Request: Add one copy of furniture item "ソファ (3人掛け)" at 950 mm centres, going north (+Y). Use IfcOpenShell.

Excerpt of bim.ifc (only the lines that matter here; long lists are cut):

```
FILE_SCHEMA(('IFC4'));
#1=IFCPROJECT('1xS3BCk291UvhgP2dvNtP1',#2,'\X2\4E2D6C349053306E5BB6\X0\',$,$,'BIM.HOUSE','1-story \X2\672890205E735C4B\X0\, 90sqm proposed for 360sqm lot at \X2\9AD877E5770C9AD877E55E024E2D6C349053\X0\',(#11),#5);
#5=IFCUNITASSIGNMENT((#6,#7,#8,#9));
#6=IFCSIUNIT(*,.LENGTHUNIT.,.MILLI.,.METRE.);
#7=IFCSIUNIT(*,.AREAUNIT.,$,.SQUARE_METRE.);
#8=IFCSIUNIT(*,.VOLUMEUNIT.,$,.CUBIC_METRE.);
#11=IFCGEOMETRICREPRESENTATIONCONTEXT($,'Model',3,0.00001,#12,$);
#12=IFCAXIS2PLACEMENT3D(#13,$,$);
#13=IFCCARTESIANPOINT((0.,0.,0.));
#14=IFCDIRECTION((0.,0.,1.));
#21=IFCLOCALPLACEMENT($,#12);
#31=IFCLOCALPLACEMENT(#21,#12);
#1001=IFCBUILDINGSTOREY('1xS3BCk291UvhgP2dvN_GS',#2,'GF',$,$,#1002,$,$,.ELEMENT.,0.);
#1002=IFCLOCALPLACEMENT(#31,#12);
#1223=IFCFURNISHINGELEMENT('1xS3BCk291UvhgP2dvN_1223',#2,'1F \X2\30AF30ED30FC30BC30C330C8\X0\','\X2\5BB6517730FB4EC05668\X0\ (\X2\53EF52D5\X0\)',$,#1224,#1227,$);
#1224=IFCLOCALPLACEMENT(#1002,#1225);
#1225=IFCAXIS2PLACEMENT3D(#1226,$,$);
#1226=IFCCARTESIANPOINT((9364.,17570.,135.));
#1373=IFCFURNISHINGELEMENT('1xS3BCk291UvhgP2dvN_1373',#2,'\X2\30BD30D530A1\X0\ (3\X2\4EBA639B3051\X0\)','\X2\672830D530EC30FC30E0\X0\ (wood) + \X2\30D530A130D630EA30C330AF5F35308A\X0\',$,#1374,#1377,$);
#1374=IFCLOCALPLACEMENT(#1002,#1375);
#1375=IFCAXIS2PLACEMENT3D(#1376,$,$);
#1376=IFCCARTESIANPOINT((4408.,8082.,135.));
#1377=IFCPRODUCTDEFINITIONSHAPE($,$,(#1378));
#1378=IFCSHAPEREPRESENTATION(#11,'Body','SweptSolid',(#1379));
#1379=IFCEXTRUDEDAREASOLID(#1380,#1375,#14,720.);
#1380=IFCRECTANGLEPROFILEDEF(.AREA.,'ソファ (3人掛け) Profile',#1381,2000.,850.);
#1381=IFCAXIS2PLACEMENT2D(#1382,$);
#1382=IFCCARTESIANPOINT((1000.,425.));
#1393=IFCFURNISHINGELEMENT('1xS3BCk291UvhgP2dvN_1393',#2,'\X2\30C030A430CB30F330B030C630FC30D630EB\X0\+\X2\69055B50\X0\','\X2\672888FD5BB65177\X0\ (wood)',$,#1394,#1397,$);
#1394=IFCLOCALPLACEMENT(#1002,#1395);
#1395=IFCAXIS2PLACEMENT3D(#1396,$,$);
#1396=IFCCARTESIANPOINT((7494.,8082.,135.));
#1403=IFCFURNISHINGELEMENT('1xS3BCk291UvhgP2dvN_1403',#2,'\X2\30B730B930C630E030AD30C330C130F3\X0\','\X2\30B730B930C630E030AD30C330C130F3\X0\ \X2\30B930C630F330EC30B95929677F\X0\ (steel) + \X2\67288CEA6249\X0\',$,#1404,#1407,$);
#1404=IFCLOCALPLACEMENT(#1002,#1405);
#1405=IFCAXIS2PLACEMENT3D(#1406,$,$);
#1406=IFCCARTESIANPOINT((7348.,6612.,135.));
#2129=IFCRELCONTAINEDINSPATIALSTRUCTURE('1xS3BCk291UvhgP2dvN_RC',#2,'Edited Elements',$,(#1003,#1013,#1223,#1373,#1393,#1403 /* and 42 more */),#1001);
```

```python
import numpy as np
import ifcopenshell
import ifcopenshell.api.geometry
import ifcopenshell.api.root
import ifcopenshell.util.element
import ifcopenshell.util.placement
import ifcopenshell.util.unit

model = ifcopenshell.open("bim.ifc")
unit_scale = ifcopenshell.util.unit.calculate_unit_scale(model)


def reuse_history(source, copy):
    """copy_class also copies each property set's owner history, people and application; keep the originals."""
    for rel in copy.IsDefinedBy:
        if rel.is_a("IfcRelDefinesByProperties") and (history := rel.RelatingPropertyDefinition.OwnerHistory):
            rel.RelatingPropertyDefinition.OwnerHistory = source.OwnerHistory
            ifcopenshell.util.element.remove_deep2(model, history)


source = model.by_guid("1xS3BCk291UvhgP2dvN_1373")
base = ifcopenshell.util.placement.get_local_placement(source.ObjectPlacement)
step = np.array([0.0, 1.0, 0.0]) * 0.95 / unit_scale

for i in range(1, 2):
    copy = ifcopenshell.api.root.copy_class(model, product=source)
    copy.Representation = ifcopenshell.util.element.copy_deep(
        model, source.Representation, exclude=["IfcGeometricRepresentationContext", "IfcRepresentationMap"]
    )
    reuse_history(source, copy)
    matrix = base.copy()
    matrix[:3, 3] += i * step
    print("added at", matrix[:3, 3].round(3) + 0.0)
    ifcopenshell.api.geometry.edit_object_placement(model, product=copy, matrix=matrix, is_si=False)

model.write("bim_updated.ifc")
```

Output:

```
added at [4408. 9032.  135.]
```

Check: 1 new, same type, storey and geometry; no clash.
